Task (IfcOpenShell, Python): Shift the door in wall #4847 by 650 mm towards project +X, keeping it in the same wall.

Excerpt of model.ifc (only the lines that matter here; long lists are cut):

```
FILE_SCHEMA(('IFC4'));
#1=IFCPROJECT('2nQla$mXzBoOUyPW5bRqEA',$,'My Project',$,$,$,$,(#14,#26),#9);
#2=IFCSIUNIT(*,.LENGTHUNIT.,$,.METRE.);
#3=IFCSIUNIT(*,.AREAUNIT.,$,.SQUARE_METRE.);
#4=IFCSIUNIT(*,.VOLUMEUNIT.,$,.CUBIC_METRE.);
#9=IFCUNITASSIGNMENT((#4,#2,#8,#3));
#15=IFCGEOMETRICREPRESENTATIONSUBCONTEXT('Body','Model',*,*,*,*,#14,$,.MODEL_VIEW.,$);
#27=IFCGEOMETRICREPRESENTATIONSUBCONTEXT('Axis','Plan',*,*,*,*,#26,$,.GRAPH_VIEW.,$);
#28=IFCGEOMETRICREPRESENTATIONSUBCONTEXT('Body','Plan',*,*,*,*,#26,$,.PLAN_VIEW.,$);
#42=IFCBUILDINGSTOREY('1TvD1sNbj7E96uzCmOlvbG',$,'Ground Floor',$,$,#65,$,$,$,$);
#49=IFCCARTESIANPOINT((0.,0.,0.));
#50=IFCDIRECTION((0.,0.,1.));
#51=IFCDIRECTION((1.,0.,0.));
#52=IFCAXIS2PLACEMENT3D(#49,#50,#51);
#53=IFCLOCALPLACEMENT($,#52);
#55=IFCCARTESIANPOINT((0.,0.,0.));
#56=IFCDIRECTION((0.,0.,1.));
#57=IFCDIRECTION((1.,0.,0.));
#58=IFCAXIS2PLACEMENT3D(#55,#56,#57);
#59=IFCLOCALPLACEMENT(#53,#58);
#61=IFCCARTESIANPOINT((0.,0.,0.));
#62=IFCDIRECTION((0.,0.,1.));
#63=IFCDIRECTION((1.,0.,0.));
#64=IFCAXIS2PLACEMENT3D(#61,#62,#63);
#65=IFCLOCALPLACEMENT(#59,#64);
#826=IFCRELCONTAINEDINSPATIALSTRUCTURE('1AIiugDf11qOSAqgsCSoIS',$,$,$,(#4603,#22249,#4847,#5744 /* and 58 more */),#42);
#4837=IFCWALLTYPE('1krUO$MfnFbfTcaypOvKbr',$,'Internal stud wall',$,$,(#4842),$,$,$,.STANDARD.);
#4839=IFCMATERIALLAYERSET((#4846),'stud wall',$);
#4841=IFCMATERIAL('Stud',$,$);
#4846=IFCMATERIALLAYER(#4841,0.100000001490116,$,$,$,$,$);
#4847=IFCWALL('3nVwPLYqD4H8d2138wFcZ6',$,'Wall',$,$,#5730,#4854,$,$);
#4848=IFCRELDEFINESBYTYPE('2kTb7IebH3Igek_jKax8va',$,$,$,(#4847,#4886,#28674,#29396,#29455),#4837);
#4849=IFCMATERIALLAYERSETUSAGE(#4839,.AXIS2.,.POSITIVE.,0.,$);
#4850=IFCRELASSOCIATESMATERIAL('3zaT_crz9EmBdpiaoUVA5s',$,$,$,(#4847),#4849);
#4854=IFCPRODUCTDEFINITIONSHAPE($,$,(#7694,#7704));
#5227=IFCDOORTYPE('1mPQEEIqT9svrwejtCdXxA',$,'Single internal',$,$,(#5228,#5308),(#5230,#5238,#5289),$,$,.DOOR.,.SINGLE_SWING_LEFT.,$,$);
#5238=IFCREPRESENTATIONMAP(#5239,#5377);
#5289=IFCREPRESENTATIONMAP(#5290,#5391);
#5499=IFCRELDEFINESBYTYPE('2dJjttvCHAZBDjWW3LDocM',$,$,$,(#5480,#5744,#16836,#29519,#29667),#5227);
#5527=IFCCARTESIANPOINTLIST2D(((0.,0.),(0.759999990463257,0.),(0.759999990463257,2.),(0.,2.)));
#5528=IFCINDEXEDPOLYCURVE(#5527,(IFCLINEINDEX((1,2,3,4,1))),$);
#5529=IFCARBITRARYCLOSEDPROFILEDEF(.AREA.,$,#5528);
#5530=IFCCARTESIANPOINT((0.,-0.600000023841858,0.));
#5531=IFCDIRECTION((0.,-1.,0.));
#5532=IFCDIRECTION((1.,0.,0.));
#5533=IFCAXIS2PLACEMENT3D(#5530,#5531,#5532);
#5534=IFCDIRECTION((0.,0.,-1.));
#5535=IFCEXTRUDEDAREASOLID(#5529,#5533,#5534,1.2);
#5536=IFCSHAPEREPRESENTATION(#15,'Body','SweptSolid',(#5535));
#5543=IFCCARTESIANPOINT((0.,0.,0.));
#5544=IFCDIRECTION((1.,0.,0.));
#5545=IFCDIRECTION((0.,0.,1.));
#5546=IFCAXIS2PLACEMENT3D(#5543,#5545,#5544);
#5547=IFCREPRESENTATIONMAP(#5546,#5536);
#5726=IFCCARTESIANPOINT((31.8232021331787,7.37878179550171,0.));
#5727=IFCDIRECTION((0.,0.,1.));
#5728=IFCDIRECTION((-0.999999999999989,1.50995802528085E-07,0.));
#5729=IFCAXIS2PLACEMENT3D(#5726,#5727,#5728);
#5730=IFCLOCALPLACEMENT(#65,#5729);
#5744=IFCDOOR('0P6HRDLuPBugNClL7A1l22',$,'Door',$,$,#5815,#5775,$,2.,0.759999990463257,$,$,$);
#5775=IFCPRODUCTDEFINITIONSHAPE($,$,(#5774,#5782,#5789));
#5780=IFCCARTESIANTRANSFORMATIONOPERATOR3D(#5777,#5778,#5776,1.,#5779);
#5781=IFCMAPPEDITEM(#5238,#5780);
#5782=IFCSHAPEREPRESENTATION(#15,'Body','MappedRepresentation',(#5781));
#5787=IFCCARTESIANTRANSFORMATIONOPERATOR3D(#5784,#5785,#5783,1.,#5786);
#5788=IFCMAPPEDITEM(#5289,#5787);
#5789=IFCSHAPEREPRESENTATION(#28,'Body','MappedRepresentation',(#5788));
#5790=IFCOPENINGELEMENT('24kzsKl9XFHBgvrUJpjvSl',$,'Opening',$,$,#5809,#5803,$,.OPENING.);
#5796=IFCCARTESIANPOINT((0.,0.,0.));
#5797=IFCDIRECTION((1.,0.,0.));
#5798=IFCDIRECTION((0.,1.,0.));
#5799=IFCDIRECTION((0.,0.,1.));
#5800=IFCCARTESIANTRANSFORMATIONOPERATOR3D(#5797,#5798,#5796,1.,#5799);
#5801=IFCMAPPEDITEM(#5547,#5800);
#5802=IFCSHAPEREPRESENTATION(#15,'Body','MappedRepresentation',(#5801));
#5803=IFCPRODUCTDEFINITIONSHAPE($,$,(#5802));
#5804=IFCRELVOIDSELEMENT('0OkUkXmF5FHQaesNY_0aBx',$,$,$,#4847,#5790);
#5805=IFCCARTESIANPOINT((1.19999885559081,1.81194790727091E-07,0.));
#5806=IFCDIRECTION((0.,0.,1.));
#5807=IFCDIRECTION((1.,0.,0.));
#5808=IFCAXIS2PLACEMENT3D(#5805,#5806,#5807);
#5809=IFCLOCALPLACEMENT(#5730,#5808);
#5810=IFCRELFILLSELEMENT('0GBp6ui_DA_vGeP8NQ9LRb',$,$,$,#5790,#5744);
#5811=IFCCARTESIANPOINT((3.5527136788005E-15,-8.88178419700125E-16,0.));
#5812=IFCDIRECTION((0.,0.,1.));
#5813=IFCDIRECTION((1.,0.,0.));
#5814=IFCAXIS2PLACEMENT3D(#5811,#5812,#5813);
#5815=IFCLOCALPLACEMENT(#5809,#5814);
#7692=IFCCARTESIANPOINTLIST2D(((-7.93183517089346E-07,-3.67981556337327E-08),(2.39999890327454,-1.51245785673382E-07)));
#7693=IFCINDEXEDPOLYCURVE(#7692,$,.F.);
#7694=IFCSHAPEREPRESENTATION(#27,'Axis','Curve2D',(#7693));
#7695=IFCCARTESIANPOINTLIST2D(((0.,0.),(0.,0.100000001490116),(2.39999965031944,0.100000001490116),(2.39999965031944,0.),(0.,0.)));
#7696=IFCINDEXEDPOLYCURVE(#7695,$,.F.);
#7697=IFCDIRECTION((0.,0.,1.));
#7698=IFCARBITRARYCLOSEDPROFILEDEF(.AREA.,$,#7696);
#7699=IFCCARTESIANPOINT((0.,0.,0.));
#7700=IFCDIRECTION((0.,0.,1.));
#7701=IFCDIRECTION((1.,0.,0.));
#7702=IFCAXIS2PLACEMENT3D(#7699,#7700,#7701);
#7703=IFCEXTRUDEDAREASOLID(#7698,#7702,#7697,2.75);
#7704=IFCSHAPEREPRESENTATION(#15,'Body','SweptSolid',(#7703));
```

```python
import ifcopenshell
import ifcopenshell.api.geometry
import ifcopenshell.util.placement
import ifcopenshell.util.unit

model = ifcopenshell.open("model.ifc")
unit_scale = ifcopenshell.util.unit.calculate_unit_scale(model)

door = model.by_guid("0P6HRDLuPBugNClL7A1l22")
opening = door.FillsVoids[0].RelatingOpeningElement
wall = opening.VoidsElements[0].RelatingBuildingElement

wall_matrix = ifcopenshell.util.placement.get_local_placement(wall.ObjectPlacement)
shift = wall_matrix[:3, 0] * -0.65 / unit_scale
before = ifcopenshell.util.placement.get_local_placement(door.ObjectPlacement)[:3, 3].copy()

# The door is placed relative to its opening, so it follows when the opening moves.
matrix = ifcopenshell.util.placement.get_local_placement(opening.ObjectPlacement)
matrix[:3, 3] += shift
ifcopenshell.api.geometry.edit_object_placement(
    model, product=opening, matrix=matrix, is_si=False, should_transform_children=True
)

after = ifcopenshell.util.placement.get_local_placement(door.ObjectPlacement)[:3, 3]
print("door moved by", (after - before).round(3) + 0.0)

model.write("model_updated.ifc")
```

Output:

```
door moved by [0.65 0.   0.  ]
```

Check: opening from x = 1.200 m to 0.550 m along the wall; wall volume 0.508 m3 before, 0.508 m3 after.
